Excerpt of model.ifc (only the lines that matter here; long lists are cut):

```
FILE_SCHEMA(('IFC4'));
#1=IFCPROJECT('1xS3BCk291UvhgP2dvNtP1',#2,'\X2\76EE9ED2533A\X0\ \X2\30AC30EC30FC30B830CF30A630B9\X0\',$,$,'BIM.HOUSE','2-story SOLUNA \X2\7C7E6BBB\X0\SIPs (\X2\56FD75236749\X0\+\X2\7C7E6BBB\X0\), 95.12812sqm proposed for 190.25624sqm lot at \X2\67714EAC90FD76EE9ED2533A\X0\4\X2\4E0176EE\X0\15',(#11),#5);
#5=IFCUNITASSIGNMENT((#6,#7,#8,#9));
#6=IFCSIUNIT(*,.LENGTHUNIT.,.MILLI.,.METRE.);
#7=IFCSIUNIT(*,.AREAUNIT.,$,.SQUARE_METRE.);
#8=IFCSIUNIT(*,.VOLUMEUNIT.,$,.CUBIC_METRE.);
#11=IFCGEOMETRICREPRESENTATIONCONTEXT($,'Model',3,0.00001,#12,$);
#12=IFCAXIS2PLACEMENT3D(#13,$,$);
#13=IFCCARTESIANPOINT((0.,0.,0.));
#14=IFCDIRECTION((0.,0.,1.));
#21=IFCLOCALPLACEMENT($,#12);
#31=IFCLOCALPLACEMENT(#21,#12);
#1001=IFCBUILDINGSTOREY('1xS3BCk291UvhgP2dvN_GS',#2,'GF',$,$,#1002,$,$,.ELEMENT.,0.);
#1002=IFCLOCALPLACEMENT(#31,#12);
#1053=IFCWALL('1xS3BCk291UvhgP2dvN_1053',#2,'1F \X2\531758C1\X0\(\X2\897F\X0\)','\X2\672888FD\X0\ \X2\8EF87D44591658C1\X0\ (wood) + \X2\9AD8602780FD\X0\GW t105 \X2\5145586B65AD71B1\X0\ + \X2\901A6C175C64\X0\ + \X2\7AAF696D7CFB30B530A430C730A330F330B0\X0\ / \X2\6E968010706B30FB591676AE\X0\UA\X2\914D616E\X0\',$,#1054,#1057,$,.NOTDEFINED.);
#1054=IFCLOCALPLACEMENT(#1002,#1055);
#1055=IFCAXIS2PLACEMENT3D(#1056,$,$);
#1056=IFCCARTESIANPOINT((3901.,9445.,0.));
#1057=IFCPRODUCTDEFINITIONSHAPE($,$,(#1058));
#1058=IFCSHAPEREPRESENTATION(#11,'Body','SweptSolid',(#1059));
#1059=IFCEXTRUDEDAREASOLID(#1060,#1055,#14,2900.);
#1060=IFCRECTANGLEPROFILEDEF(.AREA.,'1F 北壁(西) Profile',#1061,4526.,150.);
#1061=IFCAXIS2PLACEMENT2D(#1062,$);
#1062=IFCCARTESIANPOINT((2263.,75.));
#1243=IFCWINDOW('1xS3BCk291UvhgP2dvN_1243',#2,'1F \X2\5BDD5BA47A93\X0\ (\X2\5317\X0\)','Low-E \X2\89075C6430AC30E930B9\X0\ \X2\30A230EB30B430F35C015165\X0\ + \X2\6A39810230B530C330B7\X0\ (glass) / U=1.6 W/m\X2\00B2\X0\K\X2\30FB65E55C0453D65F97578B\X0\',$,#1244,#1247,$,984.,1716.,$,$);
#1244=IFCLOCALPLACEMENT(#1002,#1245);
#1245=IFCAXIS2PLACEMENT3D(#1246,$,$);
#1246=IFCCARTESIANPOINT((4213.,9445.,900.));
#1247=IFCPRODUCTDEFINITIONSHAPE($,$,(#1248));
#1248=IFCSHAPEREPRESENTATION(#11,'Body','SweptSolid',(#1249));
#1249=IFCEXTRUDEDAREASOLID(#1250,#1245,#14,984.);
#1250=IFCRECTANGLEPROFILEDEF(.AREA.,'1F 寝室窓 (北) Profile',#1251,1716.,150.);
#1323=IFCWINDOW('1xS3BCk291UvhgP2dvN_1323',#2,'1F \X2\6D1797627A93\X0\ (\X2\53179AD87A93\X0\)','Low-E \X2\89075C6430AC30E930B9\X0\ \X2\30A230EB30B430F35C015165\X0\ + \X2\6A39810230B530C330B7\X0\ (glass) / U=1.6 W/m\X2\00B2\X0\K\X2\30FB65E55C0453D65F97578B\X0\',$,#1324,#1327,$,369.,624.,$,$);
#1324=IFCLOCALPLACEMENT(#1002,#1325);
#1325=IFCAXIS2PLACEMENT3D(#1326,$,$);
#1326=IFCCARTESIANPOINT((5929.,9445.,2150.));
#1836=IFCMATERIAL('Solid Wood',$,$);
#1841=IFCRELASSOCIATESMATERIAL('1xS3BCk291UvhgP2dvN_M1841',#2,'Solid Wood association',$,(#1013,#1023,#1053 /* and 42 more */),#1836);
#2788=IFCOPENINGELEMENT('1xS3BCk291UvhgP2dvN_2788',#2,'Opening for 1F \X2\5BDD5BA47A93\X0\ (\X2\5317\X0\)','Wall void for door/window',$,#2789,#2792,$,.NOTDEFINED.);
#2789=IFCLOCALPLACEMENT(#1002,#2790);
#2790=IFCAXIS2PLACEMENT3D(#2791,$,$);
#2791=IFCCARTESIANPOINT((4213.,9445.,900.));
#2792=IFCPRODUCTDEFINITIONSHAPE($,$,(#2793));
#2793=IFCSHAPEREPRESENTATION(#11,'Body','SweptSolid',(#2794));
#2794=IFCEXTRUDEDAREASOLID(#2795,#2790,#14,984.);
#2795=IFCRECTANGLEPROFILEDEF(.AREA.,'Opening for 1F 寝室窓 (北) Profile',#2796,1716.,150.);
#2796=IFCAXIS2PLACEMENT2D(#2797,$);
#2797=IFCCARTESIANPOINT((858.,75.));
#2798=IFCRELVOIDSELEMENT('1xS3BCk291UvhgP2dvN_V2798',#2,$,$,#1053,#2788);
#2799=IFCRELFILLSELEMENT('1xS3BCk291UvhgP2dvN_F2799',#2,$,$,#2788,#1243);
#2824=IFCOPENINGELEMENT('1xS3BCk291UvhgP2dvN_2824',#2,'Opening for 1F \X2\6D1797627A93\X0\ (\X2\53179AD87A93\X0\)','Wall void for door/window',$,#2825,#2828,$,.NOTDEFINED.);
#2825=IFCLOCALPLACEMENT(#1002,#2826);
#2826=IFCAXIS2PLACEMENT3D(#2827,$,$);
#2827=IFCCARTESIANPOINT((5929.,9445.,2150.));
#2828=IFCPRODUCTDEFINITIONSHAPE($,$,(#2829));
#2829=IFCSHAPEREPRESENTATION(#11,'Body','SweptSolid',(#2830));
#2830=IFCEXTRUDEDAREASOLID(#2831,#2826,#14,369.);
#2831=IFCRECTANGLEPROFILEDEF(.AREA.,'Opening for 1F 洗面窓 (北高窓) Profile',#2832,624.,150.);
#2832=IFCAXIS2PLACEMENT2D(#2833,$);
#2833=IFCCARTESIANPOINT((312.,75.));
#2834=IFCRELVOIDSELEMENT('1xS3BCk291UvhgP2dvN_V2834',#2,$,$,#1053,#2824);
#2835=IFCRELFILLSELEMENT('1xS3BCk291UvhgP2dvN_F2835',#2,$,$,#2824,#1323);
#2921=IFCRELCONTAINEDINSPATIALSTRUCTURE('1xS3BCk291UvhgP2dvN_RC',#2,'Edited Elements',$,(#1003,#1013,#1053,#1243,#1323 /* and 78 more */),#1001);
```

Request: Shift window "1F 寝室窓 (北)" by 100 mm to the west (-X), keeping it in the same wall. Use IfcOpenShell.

```python
import ifcopenshell
import ifcopenshell.api.geometry
import ifcopenshell.util.placement
import ifcopenshell.util.unit

model = ifcopenshell.open("model.ifc")
unit_scale = ifcopenshell.util.unit.calculate_unit_scale(model)

window = model.by_guid("1xS3BCk291UvhgP2dvN_1243")
opening = window.FillsVoids[0].RelatingOpeningElement
wall = opening.VoidsElements[0].RelatingBuildingElement

wall_matrix = ifcopenshell.util.placement.get_local_placement(wall.ObjectPlacement)
shift = wall_matrix[:3, 0] * -0.1 / unit_scale
before = ifcopenshell.util.placement.get_local_placement(window.ObjectPlacement)[:3, 3].copy()

# The window is not placed relative to its opening, so move both.
for product in (opening, window):
    matrix = ifcopenshell.util.placement.get_local_placement(product.ObjectPlacement)
    matrix[:3, 3] += shift
    ifcopenshell.api.geometry.edit_object_placement(model, product=product, matrix=matrix, is_si=False)

after = ifcopenshell.util.placement.get_local_placement(window.ObjectPlacement)[:3, 3]
print("window moved by", (after - before).round(3) + 0.0)

model.write("model_edited.ifc")
```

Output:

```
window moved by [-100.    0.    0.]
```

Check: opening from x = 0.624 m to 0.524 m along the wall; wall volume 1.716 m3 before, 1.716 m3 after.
